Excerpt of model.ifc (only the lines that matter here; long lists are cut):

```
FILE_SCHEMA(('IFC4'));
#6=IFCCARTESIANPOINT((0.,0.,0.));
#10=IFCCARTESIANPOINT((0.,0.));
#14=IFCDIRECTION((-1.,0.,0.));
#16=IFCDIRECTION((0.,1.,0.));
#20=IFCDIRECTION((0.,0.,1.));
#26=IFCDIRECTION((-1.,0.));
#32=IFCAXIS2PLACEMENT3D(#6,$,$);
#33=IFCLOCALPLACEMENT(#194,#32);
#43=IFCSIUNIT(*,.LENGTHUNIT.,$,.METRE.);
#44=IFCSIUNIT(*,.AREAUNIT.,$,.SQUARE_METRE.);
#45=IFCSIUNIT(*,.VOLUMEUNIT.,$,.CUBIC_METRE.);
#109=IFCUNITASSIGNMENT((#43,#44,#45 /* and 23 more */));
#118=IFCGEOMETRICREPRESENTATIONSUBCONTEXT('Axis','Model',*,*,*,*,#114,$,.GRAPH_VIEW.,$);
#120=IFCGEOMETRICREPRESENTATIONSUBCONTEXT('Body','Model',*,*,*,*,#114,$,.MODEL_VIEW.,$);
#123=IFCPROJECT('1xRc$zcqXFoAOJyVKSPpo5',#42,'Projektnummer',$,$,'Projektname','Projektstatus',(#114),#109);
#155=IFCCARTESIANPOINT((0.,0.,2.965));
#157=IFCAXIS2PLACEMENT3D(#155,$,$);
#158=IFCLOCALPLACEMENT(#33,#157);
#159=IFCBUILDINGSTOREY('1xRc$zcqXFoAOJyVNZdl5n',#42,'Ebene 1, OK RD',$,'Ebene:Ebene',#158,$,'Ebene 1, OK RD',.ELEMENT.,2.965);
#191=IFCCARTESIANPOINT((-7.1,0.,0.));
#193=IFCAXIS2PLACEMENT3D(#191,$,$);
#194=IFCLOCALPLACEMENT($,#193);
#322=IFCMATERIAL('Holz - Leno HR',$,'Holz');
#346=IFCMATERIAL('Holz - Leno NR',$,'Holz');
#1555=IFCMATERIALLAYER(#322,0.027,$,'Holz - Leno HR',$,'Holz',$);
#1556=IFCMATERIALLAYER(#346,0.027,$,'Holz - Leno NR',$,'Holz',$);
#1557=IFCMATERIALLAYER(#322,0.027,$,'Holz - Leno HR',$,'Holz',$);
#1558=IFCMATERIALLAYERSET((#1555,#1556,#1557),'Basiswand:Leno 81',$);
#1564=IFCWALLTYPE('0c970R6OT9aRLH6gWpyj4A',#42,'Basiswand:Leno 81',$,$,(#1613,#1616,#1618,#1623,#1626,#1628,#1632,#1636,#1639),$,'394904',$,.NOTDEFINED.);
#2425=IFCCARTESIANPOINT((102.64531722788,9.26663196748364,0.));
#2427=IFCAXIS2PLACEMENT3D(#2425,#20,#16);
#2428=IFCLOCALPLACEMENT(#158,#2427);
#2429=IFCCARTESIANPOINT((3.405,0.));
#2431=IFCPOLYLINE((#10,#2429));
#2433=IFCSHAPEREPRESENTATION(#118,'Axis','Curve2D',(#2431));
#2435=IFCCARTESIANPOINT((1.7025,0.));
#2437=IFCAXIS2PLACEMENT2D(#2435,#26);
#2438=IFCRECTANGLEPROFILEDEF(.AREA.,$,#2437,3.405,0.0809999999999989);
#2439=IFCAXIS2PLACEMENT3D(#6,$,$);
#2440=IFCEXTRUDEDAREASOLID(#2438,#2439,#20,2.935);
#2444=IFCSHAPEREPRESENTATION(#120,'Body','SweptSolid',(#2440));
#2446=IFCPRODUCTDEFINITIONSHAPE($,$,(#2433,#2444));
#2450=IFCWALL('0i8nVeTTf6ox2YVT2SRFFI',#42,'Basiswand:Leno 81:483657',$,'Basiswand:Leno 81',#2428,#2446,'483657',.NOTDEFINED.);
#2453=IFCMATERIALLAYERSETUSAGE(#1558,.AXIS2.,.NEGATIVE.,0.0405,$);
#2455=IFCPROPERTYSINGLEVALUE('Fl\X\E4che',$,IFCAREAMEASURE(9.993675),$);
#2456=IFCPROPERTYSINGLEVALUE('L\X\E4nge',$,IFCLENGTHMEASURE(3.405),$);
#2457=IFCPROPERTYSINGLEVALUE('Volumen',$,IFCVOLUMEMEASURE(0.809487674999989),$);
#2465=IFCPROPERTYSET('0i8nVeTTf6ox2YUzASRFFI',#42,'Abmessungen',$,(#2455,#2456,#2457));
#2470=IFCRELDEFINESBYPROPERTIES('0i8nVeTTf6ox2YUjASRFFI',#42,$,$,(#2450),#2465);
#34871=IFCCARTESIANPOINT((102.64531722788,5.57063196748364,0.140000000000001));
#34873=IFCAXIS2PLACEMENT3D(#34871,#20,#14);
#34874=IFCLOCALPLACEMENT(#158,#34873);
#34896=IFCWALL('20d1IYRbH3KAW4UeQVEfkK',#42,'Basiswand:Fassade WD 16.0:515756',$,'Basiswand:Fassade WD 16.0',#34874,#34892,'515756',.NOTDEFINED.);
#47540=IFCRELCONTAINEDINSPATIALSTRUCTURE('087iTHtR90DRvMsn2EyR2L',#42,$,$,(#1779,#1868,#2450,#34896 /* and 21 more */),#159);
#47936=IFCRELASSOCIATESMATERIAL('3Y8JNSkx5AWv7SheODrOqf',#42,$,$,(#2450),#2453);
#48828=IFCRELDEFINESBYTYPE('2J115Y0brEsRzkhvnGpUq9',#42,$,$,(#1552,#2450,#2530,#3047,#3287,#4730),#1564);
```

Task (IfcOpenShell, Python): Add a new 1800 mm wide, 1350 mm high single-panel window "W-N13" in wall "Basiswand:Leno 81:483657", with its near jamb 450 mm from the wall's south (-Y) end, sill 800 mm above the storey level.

```python
import numpy as np
import ifcopenshell
import ifcopenshell.api.feature
import ifcopenshell.api.geometry
import ifcopenshell.api.pset
import ifcopenshell.api.root
import ifcopenshell.api.spatial
import ifcopenshell.geom
import ifcopenshell.util.element
import ifcopenshell.util.placement
import ifcopenshell.util.representation
import ifcopenshell.util.shape
import ifcopenshell.util.unit

model = ifcopenshell.open("model.ifc")
unit_scale = ifcopenshell.util.unit.calculate_unit_scale(model)
area_scale = ifcopenshell.util.unit.calculate_unit_scale(model, "AREAUNIT")
volume_scale = ifcopenshell.util.unit.calculate_unit_scale(model, "VOLUMEUNIT")
settings = ifcopenshell.geom.settings()


def volume(element):
    """Net volume in cubic metres, openings subtracted."""
    shape = ifcopenshell.geom.create_shape(settings, element)
    return ifcopenshell.util.shape.get_volume(shape.geometry)


wall = model.by_guid("0i8nVeTTf6ox2YVT2SRFFI")
storey = ifcopenshell.util.element.get_container(wall, ifc_class="IfcBuildingStorey")
context = ifcopenshell.util.representation.get_context(model, "Model", "Body", "MODEL_VIEW")
before = volume(wall)

width, height, from_end, sill = 1.8, 1.35, 0.45, 0.8  # metres

# The wall runs along its own X axis, and the end named is its -X end.
wall_shape = ifcopenshell.geom.create_shape(settings, wall)
x, y, z = ifcopenshell.util.shape.get_vertices(wall_shape.geometry).T
start = x.min() + from_end
face, thickness = float(y.min()), float(y.max() - y.min())
wall_matrix = ifcopenshell.util.placement.get_local_placement(wall.ObjectPlacement)
level = ifcopenshell.util.placement.get_local_placement(storey.ObjectPlacement)[2, 3]


def in_wall(x, y):
    """Placement at x, y metres in the wall's axes, at sill height."""
    matrix = wall_matrix.copy()
    matrix[:, 3] = wall_matrix @ np.array([x / unit_scale, y / unit_scale, 0.0, 1.0])
    matrix[2, 3] = level + sill / unit_scale
    return matrix


# Opening: a box that overshoots both wall faces by 50 mm.
opening = ifcopenshell.api.root.create_entity(model, ifc_class="IfcOpeningElement", predefined_type="OPENING")
box = ifcopenshell.api.geometry.add_wall_representation(
    model, context=context, length=width, height=height, thickness=thickness + 0.1
)
ifcopenshell.api.geometry.assign_representation(model, product=opening, representation=box)
ifcopenshell.api.geometry.edit_object_placement(model, product=opening, matrix=in_wall(start, face - 0.05), is_si=False)
ifcopenshell.api.feature.add_feature(model, feature=opening, element=wall)

window = ifcopenshell.api.root.create_entity(model, ifc_class="IfcWindow", name="W-N13", predefined_type="WINDOW")
window.OverallWidth, window.OverallHeight = width / unit_scale, height / unit_scale
window.PartitioningType = "SINGLE_PANEL"
body = ifcopenshell.api.geometry.add_window_representation(
    model,
    context=context,
    overall_width=window.OverallWidth,
    overall_height=window.OverallHeight,
    partition_type="SINGLE_PANEL",
)
ifcopenshell.api.geometry.assign_representation(model, product=window, representation=body)
ifcopenshell.api.spatial.assign_container(model, products=[window], relating_structure=storey)
ifcopenshell.api.feature.add_filling(model, opening=opening, element=window)

# Centre the window in the wall's thickness.
ifcopenshell.api.geometry.edit_object_placement(model, product=window, matrix=in_wall(start, face), is_si=False)
window_shape = ifcopenshell.geom.create_shape(settings, window)
depth = ifcopenshell.util.shape.get_vertices(window_shape.geometry)[:, 1]
offset = face + thickness / 2 - (depth.min() + depth.max()) / 2
ifcopenshell.api.geometry.edit_object_placement(model, product=window, matrix=in_wall(start, offset), is_si=False)

after = volume(wall)

# Update the wall's stored quantities.
pset = model.by_id(ifcopenshell.util.element.get_pset(wall, "Abmessungen", should_inherit=False)["id"])
ifcopenshell.api.pset.edit_pset(model, pset=pset, properties={
    "Fläche": model.create_entity("IfcAreaMeasure", after / thickness / area_scale),
    "Volumen": model.create_entity("IfcVolumeMeasure", after / volume_scale),
})

print(f"wall volume {before:.3f} -> {after:.3f} m3")

model.write("model_v2.ifc")
```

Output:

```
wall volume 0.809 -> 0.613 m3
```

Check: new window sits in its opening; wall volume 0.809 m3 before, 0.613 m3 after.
